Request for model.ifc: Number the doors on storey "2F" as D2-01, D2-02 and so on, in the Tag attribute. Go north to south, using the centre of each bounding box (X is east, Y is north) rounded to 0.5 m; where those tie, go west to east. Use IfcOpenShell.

First a look at what the model holds.

```python
import ifcopenshell
import ifcopenshell.util.element
import ifcopenshell.util.placement

model = ifcopenshell.open("model.ifc")
print(model.schema)
storey = next(s for s in model.by_type("IfcBuildingStorey") if s.Name == "2F")
doors = [e for e in ifcopenshell.util.element.get_decomposition(storey) if e.is_a("IfcDoor")]
for e in sorted(doors, key=lambda e: e.id()):
    origin = ifcopenshell.util.placement.get_local_placement(e.ObjectPlacement)[:3, 3]
    print(e.id(), e.Tag, e.Name, origin.round(2) + 0.0, sep=" | ")
```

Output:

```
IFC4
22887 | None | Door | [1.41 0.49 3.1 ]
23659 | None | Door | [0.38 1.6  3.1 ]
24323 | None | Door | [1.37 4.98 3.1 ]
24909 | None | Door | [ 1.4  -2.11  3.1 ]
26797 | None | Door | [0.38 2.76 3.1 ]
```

```python
import ifcopenshell
import ifcopenshell.geom
import ifcopenshell.util.element
import ifcopenshell.util.shape

model = ifcopenshell.open("model.ifc")
settings = ifcopenshell.geom.settings()
settings.set("use-world-coords", True)


def centre(element):
    shape = ifcopenshell.geom.create_shape(settings, element)
    return ifcopenshell.util.shape.get_bbox_centroid(shape.geometry)


storey = next(s for s in model.by_type("IfcBuildingStorey") if s.Name == "2F")
doors = [e for e in ifcopenshell.util.element.get_decomposition(storey) if e.is_a("IfcDoor")]

# Insertion points can sit at a corner or the storey origin, so sort by the geometry (in metres).
centres = {e: centre(e) for e in doors}
doors.sort(key=lambda e: (-round(centres[e][1] / 0.5), centres[e][0]))

for i, e in enumerate(doors, start=1):
    number = f"D2-{i:02d}"
    e.Tag = number
    print(e.id(), number)

model.write("model-out.ifc")
```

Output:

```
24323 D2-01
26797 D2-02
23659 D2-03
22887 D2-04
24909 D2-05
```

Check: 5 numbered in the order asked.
